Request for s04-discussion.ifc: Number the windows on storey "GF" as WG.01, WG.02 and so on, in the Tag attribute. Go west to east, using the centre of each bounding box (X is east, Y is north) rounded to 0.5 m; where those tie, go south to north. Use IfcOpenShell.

First a look at what the model holds.

```python
import ifcopenshell
import ifcopenshell.util.element
import ifcopenshell.util.placement

model = ifcopenshell.open("s04-discussion.ifc")
print(model.schema)
storey = next(s for s in model.by_type("IfcBuildingStorey") if s.Name == "GF")
windows = [e for e in ifcopenshell.util.element.get_decomposition(storey) if e.is_a("IfcWindow")]
for e in sorted(windows, key=lambda e: e.id()):
    origin = ifcopenshell.util.placement.get_local_placement(e.ObjectPlacement)[:3, 3]
    print(e.id(), e.Tag, e.Name, origin.round(2) + 0.0, sep=" | ")
```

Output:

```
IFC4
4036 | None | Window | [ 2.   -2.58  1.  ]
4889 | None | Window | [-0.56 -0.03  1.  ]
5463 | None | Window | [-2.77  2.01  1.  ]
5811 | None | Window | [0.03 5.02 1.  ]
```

```python
import ifcopenshell
import ifcopenshell.geom
import ifcopenshell.util.element
import ifcopenshell.util.shape

model = ifcopenshell.open("s04-discussion.ifc")
settings = ifcopenshell.geom.settings()
settings.set("use-world-coords", True)


def centre(element):
    shape = ifcopenshell.geom.create_shape(settings, element)
    return ifcopenshell.util.shape.get_bbox_centroid(shape.geometry)


storey = next(s for s in model.by_type("IfcBuildingStorey") if s.Name == "GF")
windows = [e for e in ifcopenshell.util.element.get_decomposition(storey) if e.is_a("IfcWindow")]

# Insertion points can sit at a corner or the storey origin, so sort by the geometry (in metres).
centres = {e: centre(e) for e in windows}
windows.sort(key=lambda e: (round(centres[e][0] / 0.5), centres[e][1]))

for i, e in enumerate(windows, start=1):
    number = f"WG.{i:02d}"
    e.Tag = number
    print(e.id(), number)

model.write("s04-discussion_v2.ifc")
```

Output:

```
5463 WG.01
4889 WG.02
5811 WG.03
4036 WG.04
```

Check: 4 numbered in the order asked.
